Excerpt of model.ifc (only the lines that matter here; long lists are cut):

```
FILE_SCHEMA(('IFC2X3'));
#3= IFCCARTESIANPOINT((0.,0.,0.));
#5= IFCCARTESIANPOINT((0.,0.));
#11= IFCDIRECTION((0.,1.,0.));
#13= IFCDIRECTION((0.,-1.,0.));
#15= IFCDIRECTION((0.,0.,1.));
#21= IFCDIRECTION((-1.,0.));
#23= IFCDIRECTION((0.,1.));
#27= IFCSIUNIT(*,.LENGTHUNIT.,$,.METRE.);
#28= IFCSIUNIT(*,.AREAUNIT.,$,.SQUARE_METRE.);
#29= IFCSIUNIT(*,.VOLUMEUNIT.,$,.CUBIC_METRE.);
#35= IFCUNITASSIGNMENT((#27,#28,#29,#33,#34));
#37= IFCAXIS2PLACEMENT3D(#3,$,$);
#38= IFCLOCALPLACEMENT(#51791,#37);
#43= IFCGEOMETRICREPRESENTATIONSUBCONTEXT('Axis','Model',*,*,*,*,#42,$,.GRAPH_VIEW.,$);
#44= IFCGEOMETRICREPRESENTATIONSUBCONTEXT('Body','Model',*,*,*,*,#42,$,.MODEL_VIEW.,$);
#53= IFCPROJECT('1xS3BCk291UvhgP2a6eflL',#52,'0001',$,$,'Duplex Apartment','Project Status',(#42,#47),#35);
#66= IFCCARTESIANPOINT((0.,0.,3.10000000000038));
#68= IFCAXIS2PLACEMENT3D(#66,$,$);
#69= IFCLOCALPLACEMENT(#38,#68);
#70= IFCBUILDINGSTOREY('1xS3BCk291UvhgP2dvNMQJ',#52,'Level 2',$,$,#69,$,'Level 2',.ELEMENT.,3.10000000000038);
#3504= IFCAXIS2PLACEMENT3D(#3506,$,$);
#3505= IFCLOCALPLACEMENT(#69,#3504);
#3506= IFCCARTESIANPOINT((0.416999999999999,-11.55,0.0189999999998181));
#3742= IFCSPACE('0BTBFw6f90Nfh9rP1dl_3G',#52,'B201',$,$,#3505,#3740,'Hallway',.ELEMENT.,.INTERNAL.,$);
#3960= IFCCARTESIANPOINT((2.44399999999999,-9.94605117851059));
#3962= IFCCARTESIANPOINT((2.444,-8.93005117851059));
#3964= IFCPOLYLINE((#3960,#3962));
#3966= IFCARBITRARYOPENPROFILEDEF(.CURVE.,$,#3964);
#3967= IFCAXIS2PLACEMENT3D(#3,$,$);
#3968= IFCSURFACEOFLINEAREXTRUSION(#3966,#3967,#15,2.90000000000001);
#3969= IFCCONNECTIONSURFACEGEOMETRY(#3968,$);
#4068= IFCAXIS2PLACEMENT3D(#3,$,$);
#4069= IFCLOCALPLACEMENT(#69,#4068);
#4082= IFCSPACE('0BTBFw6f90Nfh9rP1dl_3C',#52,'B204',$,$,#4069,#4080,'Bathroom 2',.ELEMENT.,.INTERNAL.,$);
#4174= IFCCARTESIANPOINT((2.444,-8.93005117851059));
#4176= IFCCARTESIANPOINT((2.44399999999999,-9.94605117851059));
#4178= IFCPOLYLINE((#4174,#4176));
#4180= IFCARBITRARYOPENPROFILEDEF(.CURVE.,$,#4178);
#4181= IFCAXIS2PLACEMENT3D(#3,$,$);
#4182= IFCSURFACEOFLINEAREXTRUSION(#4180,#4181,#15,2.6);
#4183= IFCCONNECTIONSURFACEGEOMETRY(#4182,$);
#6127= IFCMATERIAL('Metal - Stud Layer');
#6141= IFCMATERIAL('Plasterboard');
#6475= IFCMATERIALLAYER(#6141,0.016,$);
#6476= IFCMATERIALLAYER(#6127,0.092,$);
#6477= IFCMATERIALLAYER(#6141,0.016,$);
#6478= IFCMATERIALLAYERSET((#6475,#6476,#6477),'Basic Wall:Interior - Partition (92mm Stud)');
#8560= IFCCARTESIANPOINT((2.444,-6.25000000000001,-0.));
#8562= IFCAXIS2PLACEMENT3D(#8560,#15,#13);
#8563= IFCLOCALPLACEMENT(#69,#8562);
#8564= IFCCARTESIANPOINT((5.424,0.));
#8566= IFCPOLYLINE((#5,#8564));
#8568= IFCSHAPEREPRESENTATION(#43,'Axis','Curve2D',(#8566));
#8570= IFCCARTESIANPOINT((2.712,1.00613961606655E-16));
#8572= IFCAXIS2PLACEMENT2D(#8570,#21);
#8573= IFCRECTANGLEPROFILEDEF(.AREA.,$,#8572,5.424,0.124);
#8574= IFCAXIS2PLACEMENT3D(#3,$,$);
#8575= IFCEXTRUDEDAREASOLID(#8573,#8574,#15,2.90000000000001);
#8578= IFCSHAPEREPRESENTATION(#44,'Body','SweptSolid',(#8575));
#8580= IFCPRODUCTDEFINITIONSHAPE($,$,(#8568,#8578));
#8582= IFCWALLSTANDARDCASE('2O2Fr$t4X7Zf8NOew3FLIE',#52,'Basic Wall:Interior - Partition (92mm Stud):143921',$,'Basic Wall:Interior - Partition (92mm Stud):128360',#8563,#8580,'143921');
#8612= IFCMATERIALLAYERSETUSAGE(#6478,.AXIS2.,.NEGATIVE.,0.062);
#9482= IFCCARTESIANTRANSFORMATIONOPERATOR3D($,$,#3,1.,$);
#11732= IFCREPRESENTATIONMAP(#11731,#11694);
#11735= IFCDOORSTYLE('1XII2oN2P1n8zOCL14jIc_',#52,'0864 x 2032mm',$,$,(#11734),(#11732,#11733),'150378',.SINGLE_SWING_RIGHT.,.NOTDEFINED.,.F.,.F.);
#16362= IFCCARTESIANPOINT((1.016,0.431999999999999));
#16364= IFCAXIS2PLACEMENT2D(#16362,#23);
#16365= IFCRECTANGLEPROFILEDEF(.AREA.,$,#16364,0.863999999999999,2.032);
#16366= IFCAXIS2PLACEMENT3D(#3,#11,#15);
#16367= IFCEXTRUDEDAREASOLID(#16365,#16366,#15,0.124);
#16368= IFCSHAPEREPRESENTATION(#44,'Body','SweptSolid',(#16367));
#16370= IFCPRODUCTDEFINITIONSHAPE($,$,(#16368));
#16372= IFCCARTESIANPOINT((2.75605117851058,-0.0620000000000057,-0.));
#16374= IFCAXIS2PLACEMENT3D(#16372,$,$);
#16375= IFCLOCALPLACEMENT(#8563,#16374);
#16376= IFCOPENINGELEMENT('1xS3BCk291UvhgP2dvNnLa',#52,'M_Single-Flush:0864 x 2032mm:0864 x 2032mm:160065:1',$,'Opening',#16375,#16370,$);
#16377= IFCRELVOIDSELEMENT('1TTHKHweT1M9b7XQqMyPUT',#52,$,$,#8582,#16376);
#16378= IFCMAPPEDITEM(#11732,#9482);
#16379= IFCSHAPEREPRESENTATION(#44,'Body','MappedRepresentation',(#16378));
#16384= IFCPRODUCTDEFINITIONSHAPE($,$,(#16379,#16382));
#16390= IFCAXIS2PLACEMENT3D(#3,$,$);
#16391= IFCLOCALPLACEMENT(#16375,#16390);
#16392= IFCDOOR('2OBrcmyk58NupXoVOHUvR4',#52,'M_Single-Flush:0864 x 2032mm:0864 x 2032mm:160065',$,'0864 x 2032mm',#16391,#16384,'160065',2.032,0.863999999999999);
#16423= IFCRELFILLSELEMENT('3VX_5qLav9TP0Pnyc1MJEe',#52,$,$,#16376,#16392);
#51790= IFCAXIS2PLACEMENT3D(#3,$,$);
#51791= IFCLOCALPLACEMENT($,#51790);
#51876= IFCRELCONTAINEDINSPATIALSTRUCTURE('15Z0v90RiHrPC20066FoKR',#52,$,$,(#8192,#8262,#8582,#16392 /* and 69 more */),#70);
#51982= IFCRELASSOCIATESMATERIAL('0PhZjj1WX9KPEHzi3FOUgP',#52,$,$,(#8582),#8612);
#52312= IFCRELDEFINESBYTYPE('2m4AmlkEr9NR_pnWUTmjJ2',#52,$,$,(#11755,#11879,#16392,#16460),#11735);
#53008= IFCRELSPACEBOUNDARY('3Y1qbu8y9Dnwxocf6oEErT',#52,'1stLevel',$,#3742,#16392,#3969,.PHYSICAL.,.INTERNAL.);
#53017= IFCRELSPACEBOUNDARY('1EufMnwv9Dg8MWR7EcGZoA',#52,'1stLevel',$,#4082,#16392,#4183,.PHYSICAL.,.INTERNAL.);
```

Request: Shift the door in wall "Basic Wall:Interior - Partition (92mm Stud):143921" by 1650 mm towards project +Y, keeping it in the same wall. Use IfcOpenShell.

```python
import numpy as np
import ifcopenshell
import ifcopenshell.api.geometry
import ifcopenshell.util.placement
import ifcopenshell.util.unit

model = ifcopenshell.open("model.ifc")
unit_scale = ifcopenshell.util.unit.calculate_unit_scale(model)

door = model.by_guid("2OBrcmyk58NupXoVOHUvR4")
opening = door.FillsVoids[0].RelatingOpeningElement
wall = opening.VoidsElements[0].RelatingBuildingElement

wall_matrix = ifcopenshell.util.placement.get_local_placement(wall.ObjectPlacement)
shift = wall_matrix[:3, 0] * -1.65 / unit_scale
before = ifcopenshell.util.placement.get_local_placement(door.ObjectPlacement)[:3, 3].copy()

# The door is placed relative to its opening, so it follows when the opening moves.
matrix = ifcopenshell.util.placement.get_local_placement(opening.ObjectPlacement)
matrix[:3, 3] += shift
ifcopenshell.api.geometry.edit_object_placement(
    model, product=opening, matrix=matrix, is_si=False, should_transform_children=True
)

# Space boundary surfaces are stored in each space's coordinates; move them too.
for rel in door.ProvidesBoundaries:
    if not rel.ConnectionGeometry:
        continue
    surface = rel.ConnectionGeometry.SurfaceOnRelatingElement
    space_matrix = ifcopenshell.util.placement.get_local_placement(rel.RelatingSpace.ObjectPlacement)
    point = np.array(surface.Position.Location.Coordinates) + space_matrix[:3, :3].T @ shift
    surface.Position = model.createIfcAxis2Placement3D(
        model.createIfcCartesianPoint(point.tolist()), surface.Position.Axis, surface.Position.RefDirection
    )

after = ifcopenshell.util.placement.get_local_placement(door.ObjectPlacement)[:3, 3]
print("door moved by", (after - before).round(3) + 0.0)

model.write("model-out.ifc")
```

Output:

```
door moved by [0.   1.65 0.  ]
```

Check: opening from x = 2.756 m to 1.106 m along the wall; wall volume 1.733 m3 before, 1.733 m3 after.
